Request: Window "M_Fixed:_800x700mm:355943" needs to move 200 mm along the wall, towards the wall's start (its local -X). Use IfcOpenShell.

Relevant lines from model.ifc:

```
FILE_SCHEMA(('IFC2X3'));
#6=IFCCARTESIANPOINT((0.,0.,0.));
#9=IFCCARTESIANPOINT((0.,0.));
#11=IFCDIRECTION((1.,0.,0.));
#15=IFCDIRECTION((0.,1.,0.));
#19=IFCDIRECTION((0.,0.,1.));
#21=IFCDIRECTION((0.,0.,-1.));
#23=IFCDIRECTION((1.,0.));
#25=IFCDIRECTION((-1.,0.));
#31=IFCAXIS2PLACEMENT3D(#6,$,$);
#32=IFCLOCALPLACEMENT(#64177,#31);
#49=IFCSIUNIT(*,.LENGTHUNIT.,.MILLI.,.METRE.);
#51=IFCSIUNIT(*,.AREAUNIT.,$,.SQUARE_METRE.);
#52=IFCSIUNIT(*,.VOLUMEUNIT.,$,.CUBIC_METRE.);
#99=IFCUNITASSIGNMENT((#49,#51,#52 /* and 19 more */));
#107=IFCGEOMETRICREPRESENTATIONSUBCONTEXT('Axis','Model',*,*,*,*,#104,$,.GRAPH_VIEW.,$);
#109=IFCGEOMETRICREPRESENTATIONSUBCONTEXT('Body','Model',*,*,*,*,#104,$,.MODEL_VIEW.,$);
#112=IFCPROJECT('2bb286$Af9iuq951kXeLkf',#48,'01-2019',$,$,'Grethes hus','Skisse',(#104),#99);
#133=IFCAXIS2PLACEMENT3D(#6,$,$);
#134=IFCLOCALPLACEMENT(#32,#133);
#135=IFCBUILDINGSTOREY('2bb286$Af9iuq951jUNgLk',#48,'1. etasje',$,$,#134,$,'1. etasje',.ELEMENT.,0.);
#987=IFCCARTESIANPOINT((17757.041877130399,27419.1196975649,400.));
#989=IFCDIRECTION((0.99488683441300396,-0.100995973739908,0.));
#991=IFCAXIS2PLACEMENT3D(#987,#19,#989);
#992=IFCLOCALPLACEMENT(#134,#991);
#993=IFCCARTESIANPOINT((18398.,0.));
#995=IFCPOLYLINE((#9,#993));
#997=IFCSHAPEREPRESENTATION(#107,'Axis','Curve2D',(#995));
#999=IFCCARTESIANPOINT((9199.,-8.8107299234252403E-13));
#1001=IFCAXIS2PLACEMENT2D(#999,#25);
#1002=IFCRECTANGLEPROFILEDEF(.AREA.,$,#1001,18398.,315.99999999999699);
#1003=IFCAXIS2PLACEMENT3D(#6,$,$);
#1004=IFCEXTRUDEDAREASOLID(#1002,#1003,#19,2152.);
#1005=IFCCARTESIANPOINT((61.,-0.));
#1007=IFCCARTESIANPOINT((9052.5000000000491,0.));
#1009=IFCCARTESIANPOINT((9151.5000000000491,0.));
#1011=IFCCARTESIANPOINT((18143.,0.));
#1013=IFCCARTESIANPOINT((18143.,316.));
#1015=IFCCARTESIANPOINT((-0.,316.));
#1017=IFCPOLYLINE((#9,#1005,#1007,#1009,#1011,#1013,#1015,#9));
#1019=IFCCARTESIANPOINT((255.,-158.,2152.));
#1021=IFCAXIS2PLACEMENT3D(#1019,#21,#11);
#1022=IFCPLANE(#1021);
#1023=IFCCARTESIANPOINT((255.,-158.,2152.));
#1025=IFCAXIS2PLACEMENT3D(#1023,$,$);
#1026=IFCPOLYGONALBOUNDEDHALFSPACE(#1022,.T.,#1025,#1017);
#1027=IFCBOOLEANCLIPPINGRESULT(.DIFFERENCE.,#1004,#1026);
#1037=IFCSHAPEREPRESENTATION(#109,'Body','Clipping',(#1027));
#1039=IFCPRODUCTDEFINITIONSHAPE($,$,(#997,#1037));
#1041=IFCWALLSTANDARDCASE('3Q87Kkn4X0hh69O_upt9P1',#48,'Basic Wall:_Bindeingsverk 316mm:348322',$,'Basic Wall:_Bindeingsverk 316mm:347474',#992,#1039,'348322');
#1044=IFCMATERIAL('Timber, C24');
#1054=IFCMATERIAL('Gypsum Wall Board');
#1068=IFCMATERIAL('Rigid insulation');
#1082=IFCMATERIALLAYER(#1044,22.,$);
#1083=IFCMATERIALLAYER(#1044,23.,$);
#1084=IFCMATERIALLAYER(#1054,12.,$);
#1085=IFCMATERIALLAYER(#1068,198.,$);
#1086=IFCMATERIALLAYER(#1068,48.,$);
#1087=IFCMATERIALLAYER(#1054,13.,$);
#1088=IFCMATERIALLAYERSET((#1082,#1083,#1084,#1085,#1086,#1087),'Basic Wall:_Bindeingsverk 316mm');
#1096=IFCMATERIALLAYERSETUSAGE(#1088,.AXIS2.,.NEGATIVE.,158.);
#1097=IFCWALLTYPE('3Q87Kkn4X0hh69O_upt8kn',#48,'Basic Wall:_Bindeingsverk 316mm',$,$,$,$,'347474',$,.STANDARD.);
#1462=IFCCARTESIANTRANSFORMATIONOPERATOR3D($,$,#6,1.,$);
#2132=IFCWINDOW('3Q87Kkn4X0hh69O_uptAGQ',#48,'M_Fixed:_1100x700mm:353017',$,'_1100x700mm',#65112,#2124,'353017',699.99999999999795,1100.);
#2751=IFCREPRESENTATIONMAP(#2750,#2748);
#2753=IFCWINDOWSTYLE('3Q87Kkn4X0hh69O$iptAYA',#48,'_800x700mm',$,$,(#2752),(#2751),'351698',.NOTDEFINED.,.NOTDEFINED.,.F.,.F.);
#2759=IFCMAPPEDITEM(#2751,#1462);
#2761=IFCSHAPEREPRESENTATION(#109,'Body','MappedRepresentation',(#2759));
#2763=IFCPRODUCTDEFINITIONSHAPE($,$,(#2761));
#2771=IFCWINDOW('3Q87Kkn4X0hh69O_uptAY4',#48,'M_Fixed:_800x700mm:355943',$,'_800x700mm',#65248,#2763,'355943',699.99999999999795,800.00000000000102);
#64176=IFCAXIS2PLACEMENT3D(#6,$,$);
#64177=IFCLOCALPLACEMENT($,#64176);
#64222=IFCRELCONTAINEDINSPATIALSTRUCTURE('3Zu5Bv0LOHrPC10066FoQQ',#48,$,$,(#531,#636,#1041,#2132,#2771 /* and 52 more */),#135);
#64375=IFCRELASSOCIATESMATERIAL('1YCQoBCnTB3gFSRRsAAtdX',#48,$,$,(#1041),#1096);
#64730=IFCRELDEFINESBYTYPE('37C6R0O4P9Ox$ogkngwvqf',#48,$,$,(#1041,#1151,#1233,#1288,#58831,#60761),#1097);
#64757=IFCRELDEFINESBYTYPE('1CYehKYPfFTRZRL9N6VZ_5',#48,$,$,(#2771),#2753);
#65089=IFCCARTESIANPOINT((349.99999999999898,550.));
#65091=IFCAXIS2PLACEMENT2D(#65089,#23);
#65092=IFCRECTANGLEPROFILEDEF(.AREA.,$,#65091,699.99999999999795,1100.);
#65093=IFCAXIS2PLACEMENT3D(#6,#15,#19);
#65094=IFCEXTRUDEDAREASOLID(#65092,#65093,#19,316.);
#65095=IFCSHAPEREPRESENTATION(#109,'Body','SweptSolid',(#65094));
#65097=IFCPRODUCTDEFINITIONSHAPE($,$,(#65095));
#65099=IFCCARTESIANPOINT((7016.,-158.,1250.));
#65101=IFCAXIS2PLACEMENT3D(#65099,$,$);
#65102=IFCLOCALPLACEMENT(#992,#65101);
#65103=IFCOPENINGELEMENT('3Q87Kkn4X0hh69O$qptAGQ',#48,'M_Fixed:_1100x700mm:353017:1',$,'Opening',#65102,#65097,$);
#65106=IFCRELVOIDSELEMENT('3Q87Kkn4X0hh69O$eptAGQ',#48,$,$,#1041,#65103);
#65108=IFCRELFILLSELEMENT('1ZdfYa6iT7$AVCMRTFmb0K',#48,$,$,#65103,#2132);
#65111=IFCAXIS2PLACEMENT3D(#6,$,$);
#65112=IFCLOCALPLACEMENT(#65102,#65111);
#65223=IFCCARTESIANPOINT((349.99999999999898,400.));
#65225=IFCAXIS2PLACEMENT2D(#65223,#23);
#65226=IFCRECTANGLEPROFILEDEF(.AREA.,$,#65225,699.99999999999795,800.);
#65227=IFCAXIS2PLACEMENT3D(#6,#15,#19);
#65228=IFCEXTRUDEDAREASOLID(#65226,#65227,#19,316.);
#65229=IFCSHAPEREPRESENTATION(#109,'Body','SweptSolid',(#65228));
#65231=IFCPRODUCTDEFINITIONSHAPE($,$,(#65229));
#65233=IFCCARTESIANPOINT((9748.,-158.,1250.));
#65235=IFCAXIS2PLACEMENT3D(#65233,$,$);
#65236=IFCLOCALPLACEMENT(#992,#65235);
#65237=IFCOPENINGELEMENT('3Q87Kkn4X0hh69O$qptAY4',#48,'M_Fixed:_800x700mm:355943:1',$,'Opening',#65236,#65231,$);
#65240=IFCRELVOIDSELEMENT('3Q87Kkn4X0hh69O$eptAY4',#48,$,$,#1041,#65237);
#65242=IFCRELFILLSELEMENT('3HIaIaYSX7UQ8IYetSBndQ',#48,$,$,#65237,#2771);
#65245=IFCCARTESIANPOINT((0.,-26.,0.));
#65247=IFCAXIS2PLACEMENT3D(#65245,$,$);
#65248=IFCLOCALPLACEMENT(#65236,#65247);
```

```python
import ifcopenshell
import ifcopenshell.api.geometry
import ifcopenshell.util.placement
import ifcopenshell.util.unit

model = ifcopenshell.open("model.ifc")
unit_scale = ifcopenshell.util.unit.calculate_unit_scale(model)

window = model.by_guid("3Q87Kkn4X0hh69O_uptAY4")
opening = window.FillsVoids[0].RelatingOpeningElement
wall = opening.VoidsElements[0].RelatingBuildingElement

wall_matrix = ifcopenshell.util.placement.get_local_placement(wall.ObjectPlacement)
shift = wall_matrix[:3, 0] * -0.2 / unit_scale
before = ifcopenshell.util.placement.get_local_placement(window.ObjectPlacement)[:3, 3].copy()

# The window is placed relative to its opening, so it follows when the opening moves.
matrix = ifcopenshell.util.placement.get_local_placement(opening.ObjectPlacement)
matrix[:3, 3] += shift
ifcopenshell.api.geometry.edit_object_placement(
    model, product=opening, matrix=matrix, is_si=False, should_transform_children=True
)

after = ifcopenshell.util.placement.get_local_placement(window.ObjectPlacement)[:3, 3]
print("window moved by", (after - before).round(3) + 0.0)

model.write("model-out.ifc")
```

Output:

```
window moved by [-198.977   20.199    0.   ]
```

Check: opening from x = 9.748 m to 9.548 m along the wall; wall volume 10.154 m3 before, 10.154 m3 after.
